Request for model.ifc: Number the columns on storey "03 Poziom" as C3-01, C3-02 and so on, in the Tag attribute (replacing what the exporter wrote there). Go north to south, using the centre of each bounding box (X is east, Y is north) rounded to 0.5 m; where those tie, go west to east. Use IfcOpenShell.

First a look at what the model holds.

```python
import ifcopenshell
import ifcopenshell.util.element
import ifcopenshell.util.placement

model = ifcopenshell.open("model.ifc")
print(model.schema)
storey = next(s for s in model.by_type("IfcBuildingStorey") if s.Name == "03 Poziom")
columns = [e for e in ifcopenshell.util.element.get_decomposition(storey) if e.is_a("IfcColumn")]
for e in sorted(columns, key=lambda e: e.id()):
    origin = ifcopenshell.util.placement.get_local_placement(e.ObjectPlacement)[:3, 3]
    print(e.id(), e.Tag, e.Name, origin.round(2) + 0.0, sep=" | ")
```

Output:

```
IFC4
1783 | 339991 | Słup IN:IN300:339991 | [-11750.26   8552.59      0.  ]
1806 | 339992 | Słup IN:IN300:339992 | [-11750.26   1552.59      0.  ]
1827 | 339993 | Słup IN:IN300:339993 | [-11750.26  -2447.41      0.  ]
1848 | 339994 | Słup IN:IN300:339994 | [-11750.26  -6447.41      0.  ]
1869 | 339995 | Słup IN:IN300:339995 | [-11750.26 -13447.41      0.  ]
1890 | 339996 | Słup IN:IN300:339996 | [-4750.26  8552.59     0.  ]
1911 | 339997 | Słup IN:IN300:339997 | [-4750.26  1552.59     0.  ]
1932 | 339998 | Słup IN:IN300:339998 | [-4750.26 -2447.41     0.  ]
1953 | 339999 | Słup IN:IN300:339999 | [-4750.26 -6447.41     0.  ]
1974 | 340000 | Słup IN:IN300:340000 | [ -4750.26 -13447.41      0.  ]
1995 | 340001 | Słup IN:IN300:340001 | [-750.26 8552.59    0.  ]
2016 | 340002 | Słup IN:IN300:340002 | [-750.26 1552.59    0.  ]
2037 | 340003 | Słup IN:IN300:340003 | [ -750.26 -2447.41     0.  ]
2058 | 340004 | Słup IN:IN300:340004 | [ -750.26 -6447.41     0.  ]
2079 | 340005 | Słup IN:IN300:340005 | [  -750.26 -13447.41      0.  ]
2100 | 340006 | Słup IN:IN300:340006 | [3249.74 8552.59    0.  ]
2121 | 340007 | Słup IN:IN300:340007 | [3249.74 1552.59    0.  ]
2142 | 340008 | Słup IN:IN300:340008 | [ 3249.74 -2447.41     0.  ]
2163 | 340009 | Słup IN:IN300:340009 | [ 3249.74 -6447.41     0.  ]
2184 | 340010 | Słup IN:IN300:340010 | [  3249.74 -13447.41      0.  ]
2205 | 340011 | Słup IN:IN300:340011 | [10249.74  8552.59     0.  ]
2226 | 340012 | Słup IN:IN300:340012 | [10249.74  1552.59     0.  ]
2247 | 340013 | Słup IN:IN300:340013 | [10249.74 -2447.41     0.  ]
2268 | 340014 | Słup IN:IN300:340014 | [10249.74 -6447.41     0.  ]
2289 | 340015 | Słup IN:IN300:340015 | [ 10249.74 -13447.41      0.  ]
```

```python
import ifcopenshell
import ifcopenshell.geom
import ifcopenshell.util.element
import ifcopenshell.util.shape

model = ifcopenshell.open("model.ifc")
settings = ifcopenshell.geom.settings()
settings.set("use-world-coords", True)


def centre(element):
    shape = ifcopenshell.geom.create_shape(settings, element)
    return ifcopenshell.util.shape.get_bbox_centroid(shape.geometry)


storey = next(s for s in model.by_type("IfcBuildingStorey") if s.Name == "03 Poziom")
columns = [e for e in ifcopenshell.util.element.get_decomposition(storey) if e.is_a("IfcColumn")]

# Insertion points can sit at a corner or the storey origin, so sort by the geometry (in metres).
centres = {e: centre(e) for e in columns}
columns.sort(key=lambda e: (-round(centres[e][1] / 0.5), centres[e][0]))

for i, e in enumerate(columns, start=1):
    number = f"C3-{i:02d}"
    e.Tag = number
    print(e.id(), number)

model.write("model_rev.ifc")
```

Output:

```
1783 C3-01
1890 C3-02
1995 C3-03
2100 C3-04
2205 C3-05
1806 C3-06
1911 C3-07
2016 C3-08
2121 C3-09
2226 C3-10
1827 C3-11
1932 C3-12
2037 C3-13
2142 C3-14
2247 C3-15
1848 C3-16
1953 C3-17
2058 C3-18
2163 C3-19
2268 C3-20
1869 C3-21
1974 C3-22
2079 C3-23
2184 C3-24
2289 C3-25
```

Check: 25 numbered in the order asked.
